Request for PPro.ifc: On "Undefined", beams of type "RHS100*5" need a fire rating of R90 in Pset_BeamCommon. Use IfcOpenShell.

First a look at what the model holds.

```python
import ifcopenshell
import ifcopenshell.util.element

model = ifcopenshell.open("PPro.ifc")
print(model.schema)
storey = next(s for s in model.by_type("IfcBuildingStorey") if s.Name == "Undefined")
beams = [e for e in ifcopenshell.util.element.get_decomposition(storey) if e.is_a("IfcBeam")]
seen = {}
for e in beams:
    element_type = ifcopenshell.util.element.get_type(e)
    key = (element_type.Name if element_type != e and element_type else None, ifcopenshell.util.element.get_pset(e, "Pset_BeamCommon", "FireRating"))
    seen[key] = seen.get(key, 0) + 1
for (name, value), count in sorted(seen.items(), key=str):
    print(count, "x", name, "|", value)
```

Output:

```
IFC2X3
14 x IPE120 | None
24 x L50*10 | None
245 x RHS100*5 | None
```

```python
import ifcopenshell
import ifcopenshell.api.pset
import ifcopenshell.util.element

model = ifcopenshell.open("PPro.ifc")

storey = next(s for s in model.by_type("IfcBuildingStorey") if s.Name == "Undefined")
beams = [e for e in ifcopenshell.util.element.get_decomposition(storey) if e.is_a("IfcBeam")]

count = 0
for e in beams:
    element_type = ifcopenshell.util.element.get_type(e)
    if element_type in (None, e) or element_type.Name != "RHS100*5":
        continue
    # add_pset returns the element's existing set when there is one.
    pset = ifcopenshell.api.pset.add_pset(model, product=e, name="Pset_BeamCommon")
    ifcopenshell.api.pset.edit_pset(model, pset=pset, properties={"FireRating": "R90"})
    count += 1

print(count, "beams updated")

model.write("PPro-out.ifc")
```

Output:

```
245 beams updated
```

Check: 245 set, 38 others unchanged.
